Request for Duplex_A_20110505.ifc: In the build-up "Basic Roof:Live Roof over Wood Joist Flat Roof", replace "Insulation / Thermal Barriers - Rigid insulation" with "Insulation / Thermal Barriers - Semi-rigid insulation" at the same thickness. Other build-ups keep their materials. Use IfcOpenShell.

First a look at what the model holds.

```python
import ifcopenshell
import ifcopenshell.util.element

model = ifcopenshell.open("Duplex_A_20110505.ifc")
print(model.schema)
for layer_set in model.by_type("IfcMaterialLayerSet"):
    if layer_set.LayerSetName == "Basic Roof:Live Roof over Wood Joist Flat Roof":
        for layer in layer_set.MaterialLayers:
            print(layer.id(), layer.Material and layer.Material.Name, layer.LayerThickness, sep=" | ")
        print(len(ifcopenshell.util.element.get_elements_by_material(model, layer_set)), "elements and types use it")
print(sorted(m.Name for m in model.by_type("IfcMaterial") if m.Name)[:60])
```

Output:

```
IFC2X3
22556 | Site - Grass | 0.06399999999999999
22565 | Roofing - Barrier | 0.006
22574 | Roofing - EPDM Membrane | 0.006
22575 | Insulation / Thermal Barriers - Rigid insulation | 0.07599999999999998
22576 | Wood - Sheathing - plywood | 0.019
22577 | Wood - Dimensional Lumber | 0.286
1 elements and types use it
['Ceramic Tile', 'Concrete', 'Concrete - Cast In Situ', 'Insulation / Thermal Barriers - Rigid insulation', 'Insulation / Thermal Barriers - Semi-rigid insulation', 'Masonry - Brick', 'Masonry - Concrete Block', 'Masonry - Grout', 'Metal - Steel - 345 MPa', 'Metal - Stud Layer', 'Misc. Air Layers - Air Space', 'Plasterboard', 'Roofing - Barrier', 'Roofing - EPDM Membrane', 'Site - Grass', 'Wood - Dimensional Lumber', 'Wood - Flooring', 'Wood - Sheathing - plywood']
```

```python
import ifcopenshell
import ifcopenshell.api.material

model = ifcopenshell.open("Duplex_A_20110505.ifc")

layer_set = next(s for s in model.by_type("IfcMaterialLayerSet") if s.LayerSetName == "Basic Roof:Live Roof over Wood Joist Flat Roof")
layer = next(l for l in layer_set.MaterialLayers if l.Material and l.Material.Name == "Insulation / Thermal Barriers - Rigid insulation")
material = next(m for m in model.by_type("IfcMaterial") if m.Name == "Insulation / Thermal Barriers - Semi-rigid insulation")

# Point this one layer at the other material; renaming the old one would change it everywhere.
ifcopenshell.api.material.edit_layer(model, layer=layer, attributes={}, material=material)

print([l.Material.Name if l.Material else None for l in layer_set.MaterialLayers])

model.write("Duplex_A_20110505_edited.ifc")
```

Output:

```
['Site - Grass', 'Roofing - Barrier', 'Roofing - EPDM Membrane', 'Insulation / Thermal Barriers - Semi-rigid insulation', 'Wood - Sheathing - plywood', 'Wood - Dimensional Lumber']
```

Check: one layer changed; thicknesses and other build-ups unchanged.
